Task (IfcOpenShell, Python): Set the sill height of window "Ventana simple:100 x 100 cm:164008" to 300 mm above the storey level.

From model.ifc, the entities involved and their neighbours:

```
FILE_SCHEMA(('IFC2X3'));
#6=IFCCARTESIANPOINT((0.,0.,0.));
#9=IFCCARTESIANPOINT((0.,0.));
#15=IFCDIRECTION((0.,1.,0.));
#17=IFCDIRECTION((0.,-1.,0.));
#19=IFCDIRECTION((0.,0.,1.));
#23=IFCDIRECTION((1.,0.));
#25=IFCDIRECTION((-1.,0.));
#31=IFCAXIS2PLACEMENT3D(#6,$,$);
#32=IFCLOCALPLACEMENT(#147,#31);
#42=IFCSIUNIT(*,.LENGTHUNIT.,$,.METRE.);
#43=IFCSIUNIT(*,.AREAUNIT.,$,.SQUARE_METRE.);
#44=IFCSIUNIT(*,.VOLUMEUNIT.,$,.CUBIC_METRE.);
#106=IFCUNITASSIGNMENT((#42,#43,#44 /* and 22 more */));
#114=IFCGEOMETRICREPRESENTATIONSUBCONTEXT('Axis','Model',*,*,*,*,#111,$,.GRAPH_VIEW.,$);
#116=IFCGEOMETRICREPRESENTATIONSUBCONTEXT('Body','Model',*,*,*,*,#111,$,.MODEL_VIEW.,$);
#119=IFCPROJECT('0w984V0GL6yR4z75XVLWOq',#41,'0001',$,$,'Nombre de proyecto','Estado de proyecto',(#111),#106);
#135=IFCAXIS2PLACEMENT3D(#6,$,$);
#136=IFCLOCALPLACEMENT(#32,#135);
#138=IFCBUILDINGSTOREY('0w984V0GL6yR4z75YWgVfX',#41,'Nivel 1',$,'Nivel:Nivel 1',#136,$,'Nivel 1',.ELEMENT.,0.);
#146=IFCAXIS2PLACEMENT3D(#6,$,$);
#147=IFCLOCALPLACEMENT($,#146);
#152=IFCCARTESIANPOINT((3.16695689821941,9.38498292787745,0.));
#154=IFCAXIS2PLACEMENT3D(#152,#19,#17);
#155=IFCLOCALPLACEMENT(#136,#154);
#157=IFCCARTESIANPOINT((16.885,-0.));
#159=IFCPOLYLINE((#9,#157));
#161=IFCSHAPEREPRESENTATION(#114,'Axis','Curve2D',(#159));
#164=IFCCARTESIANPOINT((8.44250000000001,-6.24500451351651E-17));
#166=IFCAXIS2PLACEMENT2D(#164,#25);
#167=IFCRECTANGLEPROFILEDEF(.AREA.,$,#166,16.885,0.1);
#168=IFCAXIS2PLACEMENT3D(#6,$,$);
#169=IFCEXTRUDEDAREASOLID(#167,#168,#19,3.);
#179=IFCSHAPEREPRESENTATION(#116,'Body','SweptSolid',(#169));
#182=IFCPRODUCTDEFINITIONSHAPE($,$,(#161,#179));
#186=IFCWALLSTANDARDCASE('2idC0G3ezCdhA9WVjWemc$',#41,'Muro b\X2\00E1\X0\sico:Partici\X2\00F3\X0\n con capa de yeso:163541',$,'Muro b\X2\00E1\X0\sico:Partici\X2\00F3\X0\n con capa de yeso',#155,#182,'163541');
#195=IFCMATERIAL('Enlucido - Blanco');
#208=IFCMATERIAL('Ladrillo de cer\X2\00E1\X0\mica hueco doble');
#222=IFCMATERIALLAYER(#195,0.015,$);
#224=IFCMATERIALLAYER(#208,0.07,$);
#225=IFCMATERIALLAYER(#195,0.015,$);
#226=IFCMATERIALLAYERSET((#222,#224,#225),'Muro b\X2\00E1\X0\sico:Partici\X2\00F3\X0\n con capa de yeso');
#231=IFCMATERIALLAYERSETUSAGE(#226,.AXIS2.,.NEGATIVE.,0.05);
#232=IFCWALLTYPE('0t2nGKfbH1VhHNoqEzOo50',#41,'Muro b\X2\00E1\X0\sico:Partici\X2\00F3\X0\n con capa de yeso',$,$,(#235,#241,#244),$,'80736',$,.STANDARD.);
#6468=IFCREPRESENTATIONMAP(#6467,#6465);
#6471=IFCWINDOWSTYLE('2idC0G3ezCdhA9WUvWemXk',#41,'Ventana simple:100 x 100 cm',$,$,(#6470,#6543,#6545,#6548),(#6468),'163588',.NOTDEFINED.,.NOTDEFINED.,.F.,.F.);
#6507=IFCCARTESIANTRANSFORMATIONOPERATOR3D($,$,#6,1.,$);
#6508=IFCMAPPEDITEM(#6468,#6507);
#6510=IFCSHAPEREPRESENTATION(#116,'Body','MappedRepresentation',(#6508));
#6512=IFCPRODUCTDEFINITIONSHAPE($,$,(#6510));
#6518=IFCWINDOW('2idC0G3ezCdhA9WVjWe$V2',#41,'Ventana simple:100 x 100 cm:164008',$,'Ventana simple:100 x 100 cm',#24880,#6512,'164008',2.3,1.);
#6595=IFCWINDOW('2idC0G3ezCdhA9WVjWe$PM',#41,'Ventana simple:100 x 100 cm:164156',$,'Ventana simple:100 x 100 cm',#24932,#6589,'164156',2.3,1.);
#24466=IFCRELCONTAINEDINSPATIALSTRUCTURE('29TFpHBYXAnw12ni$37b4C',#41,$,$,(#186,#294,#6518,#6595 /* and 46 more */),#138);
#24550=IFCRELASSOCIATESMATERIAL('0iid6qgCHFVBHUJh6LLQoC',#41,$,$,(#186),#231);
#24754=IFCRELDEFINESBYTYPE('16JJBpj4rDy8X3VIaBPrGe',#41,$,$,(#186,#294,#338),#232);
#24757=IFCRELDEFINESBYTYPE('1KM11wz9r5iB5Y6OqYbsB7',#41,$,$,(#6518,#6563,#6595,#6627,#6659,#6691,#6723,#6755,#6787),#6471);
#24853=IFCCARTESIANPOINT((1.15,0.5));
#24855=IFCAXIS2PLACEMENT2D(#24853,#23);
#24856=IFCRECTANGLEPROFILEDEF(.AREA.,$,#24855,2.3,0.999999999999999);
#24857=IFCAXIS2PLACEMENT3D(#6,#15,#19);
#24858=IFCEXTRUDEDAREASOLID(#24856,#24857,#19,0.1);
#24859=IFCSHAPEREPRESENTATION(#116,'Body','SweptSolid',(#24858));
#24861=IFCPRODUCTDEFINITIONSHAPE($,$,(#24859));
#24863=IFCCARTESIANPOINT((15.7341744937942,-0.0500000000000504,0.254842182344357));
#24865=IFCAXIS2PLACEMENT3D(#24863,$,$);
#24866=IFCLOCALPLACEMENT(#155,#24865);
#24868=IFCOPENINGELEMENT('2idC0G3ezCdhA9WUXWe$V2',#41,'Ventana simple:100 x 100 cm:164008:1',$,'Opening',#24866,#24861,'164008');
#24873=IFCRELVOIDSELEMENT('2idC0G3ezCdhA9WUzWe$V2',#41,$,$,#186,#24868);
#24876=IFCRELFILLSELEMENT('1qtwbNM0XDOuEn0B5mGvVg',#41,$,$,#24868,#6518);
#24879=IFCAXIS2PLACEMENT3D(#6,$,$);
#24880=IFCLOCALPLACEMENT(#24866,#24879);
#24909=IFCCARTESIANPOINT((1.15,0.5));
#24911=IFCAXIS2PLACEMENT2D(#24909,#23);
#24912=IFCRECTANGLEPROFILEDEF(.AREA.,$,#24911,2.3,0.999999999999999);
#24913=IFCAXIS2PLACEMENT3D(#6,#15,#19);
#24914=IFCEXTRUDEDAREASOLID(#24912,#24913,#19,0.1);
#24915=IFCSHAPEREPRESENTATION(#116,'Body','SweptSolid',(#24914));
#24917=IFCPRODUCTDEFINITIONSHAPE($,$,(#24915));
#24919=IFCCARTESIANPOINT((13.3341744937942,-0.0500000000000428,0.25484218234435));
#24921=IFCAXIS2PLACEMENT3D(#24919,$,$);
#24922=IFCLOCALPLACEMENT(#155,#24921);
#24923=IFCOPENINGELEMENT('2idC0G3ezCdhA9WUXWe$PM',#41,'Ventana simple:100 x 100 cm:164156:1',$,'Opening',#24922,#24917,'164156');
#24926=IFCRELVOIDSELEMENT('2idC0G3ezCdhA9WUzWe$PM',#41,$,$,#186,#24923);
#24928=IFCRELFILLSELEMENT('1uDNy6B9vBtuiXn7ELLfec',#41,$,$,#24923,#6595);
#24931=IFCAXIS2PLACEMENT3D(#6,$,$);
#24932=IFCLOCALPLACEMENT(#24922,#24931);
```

```python
import numpy as np
import ifcopenshell
import ifcopenshell.api.geometry
import ifcopenshell.geom
import ifcopenshell.util.element
import ifcopenshell.util.placement
import ifcopenshell.util.shape
import ifcopenshell.util.unit

model = ifcopenshell.open("model.ifc")
unit_scale = ifcopenshell.util.unit.calculate_unit_scale(model)

window = model.by_guid("2idC0G3ezCdhA9WVjWe$V2")
opening = window.FillsVoids[0].RelatingOpeningElement
storey = ifcopenshell.util.element.get_container(window, ifc_class="IfcBuildingStorey")
level = ifcopenshell.util.placement.get_local_placement(storey.ObjectPlacement)[2, 3]

# The opening's origin need not be at the sill, so measure its lowest point.
shape = ifcopenshell.geom.create_shape(ifcopenshell.geom.settings(), opening)
bottom = ifcopenshell.util.shape.get_shape_bottom_elevation(shape, shape.geometry) / unit_scale
dz = level + 0.3 - bottom

shift = np.array([0.0, 0.0, dz])
# The window is placed relative to its opening, so it follows when the opening moves.
matrix = ifcopenshell.util.placement.get_local_placement(opening.ObjectPlacement)
matrix[:3, 3] += shift
ifcopenshell.api.geometry.edit_object_placement(
    model, product=opening, matrix=matrix, is_si=False, should_transform_children=True
)

print(f"moved by {dz * unit_scale:+.3f} m")

model.write("model_rev.ifc")
```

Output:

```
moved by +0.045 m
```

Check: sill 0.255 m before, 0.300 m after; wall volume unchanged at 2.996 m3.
